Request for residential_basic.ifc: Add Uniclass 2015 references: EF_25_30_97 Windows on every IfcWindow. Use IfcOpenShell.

First a look at what the model holds.

```python
import ifcopenshell

model = ifcopenshell.open("residential_basic.ifc")
print(model.schema)
print("classifications:", [c.Name for c in model.by_type("IfcClassification")])
for ifc_class in ("IfcDoor", "IfcRoof", "IfcStair", "IfcWall", "IfcWindow"):
    print(ifc_class, len(model.by_type(ifc_class)))
```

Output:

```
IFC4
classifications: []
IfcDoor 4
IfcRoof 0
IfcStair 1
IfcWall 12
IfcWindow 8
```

```python
import ifcopenshell
import ifcopenshell.api.classification

model = ifcopenshell.open("residential_basic.ifc")

system = ifcopenshell.api.classification.add_classification(model, classification="Uniclass 2015")

codes = {
    "IfcWindow": ("EF_25_30_97", "Windows"),
}
for ifc_class, (code, name) in codes.items():
    products = model.by_type(ifc_class)
    ifcopenshell.api.classification.add_reference(
        model, products=products, classification=system, identification=code, name=name
    )
    print(code, len(products))

model.write("residential_basic-out.ifc")
```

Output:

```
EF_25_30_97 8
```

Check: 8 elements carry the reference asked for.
